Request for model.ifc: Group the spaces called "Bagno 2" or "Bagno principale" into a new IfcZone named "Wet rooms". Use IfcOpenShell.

First a look at what the model holds.

```python
import ifcopenshell

model = ifcopenshell.open("model.ifc")
print(model.schema)
seen = {}
for space in model.by_type("IfcSpace"):
    seen[space.LongName] = seen.get(space.LongName, 0) + 1
for name, count in sorted(seen.items(), key=str):
    print(count, "x", name)
print("zones:", [z.Name for z in model.by_type("IfcZone")][:20])
```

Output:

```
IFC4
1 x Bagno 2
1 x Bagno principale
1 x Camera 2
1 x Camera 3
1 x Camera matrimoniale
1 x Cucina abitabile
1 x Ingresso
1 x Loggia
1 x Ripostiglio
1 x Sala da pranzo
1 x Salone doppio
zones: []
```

```python
import ifcopenshell
import ifcopenshell.api.group
import ifcopenshell.api.root

model = ifcopenshell.open("model.ifc")

names = {"Bagno 2", "Bagno principale"}
spaces = [s for s in model.by_type("IfcSpace") if s.LongName in names]

zone = ifcopenshell.api.root.create_entity(model, ifc_class="IfcZone", name="Wet rooms")
ifcopenshell.api.group.assign_group(model, products=spaces, group=zone)
print(len(spaces), "spaces in", zone.Name)

model.write("model_edited.ifc")
```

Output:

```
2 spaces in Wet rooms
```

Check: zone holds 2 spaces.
